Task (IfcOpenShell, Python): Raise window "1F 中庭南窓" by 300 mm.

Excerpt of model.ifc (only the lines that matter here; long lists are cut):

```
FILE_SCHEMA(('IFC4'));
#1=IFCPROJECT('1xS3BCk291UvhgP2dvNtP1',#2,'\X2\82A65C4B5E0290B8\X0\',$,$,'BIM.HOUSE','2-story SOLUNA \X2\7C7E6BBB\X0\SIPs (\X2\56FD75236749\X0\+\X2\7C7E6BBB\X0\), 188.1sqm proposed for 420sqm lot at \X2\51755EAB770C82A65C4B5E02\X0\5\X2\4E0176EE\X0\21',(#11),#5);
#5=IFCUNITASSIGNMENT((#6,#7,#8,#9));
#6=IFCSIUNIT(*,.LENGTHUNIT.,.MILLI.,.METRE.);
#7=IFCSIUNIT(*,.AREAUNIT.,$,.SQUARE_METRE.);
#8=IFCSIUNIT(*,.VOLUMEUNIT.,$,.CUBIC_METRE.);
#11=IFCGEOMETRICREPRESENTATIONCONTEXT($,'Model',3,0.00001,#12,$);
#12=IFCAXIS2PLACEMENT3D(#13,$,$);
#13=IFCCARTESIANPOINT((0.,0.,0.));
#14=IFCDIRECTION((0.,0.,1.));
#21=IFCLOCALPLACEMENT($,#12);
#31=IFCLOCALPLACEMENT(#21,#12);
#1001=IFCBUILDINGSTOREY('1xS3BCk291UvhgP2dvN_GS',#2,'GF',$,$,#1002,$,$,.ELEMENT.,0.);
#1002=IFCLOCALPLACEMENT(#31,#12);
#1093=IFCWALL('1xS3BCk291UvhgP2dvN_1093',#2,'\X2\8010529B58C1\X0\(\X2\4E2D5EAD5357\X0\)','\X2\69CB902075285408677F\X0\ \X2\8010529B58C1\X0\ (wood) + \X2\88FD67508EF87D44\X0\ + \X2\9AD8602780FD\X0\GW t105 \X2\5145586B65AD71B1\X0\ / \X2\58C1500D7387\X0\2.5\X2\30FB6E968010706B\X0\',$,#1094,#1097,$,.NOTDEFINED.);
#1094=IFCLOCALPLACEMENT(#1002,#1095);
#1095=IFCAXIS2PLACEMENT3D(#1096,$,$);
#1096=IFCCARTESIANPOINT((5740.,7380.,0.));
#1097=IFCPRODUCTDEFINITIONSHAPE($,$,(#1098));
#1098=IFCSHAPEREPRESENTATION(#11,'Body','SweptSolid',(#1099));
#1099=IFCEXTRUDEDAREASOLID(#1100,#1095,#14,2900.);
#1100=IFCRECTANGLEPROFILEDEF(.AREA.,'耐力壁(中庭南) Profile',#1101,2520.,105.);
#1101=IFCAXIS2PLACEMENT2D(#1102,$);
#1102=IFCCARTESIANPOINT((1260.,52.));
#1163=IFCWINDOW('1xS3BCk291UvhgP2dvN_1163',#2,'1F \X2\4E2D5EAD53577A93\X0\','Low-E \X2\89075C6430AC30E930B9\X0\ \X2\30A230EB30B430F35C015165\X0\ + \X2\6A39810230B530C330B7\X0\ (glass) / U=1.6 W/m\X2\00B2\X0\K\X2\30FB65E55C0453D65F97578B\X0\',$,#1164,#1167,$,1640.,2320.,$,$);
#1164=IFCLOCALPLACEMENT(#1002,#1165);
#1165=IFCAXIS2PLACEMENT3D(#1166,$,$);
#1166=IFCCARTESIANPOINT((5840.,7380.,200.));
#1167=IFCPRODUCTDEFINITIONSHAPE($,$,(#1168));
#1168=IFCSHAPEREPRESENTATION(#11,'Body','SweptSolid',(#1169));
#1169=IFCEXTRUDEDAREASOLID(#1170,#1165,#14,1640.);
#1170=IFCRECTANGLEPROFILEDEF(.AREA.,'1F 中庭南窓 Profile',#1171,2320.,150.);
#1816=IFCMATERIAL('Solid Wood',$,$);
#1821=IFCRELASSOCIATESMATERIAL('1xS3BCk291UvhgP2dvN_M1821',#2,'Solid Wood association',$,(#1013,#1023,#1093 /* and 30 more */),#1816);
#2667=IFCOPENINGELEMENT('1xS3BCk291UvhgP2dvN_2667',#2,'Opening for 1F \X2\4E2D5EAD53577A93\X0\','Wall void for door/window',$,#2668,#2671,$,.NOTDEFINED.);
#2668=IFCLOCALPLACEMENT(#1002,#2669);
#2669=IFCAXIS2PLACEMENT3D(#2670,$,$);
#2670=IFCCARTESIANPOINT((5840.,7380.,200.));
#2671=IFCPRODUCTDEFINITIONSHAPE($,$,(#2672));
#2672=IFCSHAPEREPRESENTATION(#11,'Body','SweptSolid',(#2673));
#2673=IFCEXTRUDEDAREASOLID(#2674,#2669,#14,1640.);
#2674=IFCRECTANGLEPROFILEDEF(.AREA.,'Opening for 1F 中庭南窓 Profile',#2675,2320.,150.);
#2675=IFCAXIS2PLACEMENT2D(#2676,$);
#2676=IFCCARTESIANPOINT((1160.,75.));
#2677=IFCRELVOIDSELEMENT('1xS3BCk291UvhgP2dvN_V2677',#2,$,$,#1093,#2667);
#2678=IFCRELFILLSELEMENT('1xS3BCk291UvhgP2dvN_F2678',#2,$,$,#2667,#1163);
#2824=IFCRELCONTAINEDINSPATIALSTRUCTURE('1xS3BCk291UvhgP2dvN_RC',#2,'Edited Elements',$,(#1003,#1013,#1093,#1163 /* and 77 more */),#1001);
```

```python
import numpy as np
import ifcopenshell
import ifcopenshell.api.geometry
import ifcopenshell.util.placement
import ifcopenshell.util.unit

model = ifcopenshell.open("model.ifc")
unit_scale = ifcopenshell.util.unit.calculate_unit_scale(model)

window = model.by_guid("1xS3BCk291UvhgP2dvN_1163")
opening = window.FillsVoids[0].RelatingOpeningElement
dz = 300.0

shift = np.array([0.0, 0.0, dz])
# The window is not placed relative to its opening, so move both.
for product in (opening, window):
    matrix = ifcopenshell.util.placement.get_local_placement(product.ObjectPlacement)
    matrix[:3, 3] += shift
    ifcopenshell.api.geometry.edit_object_placement(model, product=product, matrix=matrix, is_si=False)

print(f"moved by {dz * unit_scale:+.3f} m")

model.write("model_v2.ifc")
```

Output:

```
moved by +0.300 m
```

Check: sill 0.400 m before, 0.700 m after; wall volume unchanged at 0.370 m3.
